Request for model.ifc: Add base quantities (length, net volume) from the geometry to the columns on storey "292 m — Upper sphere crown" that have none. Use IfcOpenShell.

First a look at what the model holds.

```python
import ifcopenshell
import ifcopenshell.util.element
import ifcopenshell.util.unit

model = ifcopenshell.open("model.ifc")
print(model.schema)
for unit_type in ("LENGTHUNIT", "AREAUNIT", "VOLUMEUNIT"):
    print(unit_type, ifcopenshell.util.unit.calculate_unit_scale(model, unit_type))
storey = next(s for s in model.by_type("IfcBuildingStorey") if s.Name == "292 m — Upper sphere crown")
columns = [e for e in ifcopenshell.util.element.get_decomposition(storey) if e.is_a("IfcColumn")]
for e in sorted(columns, key=lambda e: e.id()):
    print(e.id(), e.is_a(), e.Name, list(ifcopenshell.util.element.get_psets(e, qtos_only=True)), sep=" | ")
```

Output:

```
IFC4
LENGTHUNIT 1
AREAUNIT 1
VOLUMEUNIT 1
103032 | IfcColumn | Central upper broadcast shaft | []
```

```python
import ifcopenshell
import ifcopenshell.api.pset
import ifcopenshell.geom
import ifcopenshell.util.element
import ifcopenshell.util.shape
import ifcopenshell.util.unit

model = ifcopenshell.open("model.ifc")
unit_scale = ifcopenshell.util.unit.calculate_unit_scale(model)
volume_scale = ifcopenshell.util.unit.calculate_unit_scale(model, "VOLUMEUNIT")
settings = ifcopenshell.geom.settings()

storey = next(s for s in model.by_type("IfcBuildingStorey") if s.Name == "292 m — Upper sphere crown")
columns = [e for e in ifcopenshell.util.element.get_decomposition(storey) if e.is_a("IfcColumn")]

for e in sorted(columns, key=lambda e: e.id()):
    if ifcopenshell.util.element.get_psets(e, qtos_only=True, should_inherit=False):
        continue
    # Geometry comes back in metres, in the element's own axes.
    shape = ifcopenshell.geom.create_shape(settings, e)
    values = {
        "Length": ifcopenshell.util.shape.get_z(shape.geometry) / unit_scale,
        "NetVolume": ifcopenshell.util.shape.get_volume(shape.geometry) / volume_scale,
    }
    qto = ifcopenshell.api.pset.add_qto(model, product=e, name="Qto_ColumnBaseQuantities")
    ifcopenshell.api.pset.edit_qto(model, qto=qto, properties=values)
    print(e.id(), {k: round(v, 3) for k, v in values.items()})

model.write("model_rev.ifc")
```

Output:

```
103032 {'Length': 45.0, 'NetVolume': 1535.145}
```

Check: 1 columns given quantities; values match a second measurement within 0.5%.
